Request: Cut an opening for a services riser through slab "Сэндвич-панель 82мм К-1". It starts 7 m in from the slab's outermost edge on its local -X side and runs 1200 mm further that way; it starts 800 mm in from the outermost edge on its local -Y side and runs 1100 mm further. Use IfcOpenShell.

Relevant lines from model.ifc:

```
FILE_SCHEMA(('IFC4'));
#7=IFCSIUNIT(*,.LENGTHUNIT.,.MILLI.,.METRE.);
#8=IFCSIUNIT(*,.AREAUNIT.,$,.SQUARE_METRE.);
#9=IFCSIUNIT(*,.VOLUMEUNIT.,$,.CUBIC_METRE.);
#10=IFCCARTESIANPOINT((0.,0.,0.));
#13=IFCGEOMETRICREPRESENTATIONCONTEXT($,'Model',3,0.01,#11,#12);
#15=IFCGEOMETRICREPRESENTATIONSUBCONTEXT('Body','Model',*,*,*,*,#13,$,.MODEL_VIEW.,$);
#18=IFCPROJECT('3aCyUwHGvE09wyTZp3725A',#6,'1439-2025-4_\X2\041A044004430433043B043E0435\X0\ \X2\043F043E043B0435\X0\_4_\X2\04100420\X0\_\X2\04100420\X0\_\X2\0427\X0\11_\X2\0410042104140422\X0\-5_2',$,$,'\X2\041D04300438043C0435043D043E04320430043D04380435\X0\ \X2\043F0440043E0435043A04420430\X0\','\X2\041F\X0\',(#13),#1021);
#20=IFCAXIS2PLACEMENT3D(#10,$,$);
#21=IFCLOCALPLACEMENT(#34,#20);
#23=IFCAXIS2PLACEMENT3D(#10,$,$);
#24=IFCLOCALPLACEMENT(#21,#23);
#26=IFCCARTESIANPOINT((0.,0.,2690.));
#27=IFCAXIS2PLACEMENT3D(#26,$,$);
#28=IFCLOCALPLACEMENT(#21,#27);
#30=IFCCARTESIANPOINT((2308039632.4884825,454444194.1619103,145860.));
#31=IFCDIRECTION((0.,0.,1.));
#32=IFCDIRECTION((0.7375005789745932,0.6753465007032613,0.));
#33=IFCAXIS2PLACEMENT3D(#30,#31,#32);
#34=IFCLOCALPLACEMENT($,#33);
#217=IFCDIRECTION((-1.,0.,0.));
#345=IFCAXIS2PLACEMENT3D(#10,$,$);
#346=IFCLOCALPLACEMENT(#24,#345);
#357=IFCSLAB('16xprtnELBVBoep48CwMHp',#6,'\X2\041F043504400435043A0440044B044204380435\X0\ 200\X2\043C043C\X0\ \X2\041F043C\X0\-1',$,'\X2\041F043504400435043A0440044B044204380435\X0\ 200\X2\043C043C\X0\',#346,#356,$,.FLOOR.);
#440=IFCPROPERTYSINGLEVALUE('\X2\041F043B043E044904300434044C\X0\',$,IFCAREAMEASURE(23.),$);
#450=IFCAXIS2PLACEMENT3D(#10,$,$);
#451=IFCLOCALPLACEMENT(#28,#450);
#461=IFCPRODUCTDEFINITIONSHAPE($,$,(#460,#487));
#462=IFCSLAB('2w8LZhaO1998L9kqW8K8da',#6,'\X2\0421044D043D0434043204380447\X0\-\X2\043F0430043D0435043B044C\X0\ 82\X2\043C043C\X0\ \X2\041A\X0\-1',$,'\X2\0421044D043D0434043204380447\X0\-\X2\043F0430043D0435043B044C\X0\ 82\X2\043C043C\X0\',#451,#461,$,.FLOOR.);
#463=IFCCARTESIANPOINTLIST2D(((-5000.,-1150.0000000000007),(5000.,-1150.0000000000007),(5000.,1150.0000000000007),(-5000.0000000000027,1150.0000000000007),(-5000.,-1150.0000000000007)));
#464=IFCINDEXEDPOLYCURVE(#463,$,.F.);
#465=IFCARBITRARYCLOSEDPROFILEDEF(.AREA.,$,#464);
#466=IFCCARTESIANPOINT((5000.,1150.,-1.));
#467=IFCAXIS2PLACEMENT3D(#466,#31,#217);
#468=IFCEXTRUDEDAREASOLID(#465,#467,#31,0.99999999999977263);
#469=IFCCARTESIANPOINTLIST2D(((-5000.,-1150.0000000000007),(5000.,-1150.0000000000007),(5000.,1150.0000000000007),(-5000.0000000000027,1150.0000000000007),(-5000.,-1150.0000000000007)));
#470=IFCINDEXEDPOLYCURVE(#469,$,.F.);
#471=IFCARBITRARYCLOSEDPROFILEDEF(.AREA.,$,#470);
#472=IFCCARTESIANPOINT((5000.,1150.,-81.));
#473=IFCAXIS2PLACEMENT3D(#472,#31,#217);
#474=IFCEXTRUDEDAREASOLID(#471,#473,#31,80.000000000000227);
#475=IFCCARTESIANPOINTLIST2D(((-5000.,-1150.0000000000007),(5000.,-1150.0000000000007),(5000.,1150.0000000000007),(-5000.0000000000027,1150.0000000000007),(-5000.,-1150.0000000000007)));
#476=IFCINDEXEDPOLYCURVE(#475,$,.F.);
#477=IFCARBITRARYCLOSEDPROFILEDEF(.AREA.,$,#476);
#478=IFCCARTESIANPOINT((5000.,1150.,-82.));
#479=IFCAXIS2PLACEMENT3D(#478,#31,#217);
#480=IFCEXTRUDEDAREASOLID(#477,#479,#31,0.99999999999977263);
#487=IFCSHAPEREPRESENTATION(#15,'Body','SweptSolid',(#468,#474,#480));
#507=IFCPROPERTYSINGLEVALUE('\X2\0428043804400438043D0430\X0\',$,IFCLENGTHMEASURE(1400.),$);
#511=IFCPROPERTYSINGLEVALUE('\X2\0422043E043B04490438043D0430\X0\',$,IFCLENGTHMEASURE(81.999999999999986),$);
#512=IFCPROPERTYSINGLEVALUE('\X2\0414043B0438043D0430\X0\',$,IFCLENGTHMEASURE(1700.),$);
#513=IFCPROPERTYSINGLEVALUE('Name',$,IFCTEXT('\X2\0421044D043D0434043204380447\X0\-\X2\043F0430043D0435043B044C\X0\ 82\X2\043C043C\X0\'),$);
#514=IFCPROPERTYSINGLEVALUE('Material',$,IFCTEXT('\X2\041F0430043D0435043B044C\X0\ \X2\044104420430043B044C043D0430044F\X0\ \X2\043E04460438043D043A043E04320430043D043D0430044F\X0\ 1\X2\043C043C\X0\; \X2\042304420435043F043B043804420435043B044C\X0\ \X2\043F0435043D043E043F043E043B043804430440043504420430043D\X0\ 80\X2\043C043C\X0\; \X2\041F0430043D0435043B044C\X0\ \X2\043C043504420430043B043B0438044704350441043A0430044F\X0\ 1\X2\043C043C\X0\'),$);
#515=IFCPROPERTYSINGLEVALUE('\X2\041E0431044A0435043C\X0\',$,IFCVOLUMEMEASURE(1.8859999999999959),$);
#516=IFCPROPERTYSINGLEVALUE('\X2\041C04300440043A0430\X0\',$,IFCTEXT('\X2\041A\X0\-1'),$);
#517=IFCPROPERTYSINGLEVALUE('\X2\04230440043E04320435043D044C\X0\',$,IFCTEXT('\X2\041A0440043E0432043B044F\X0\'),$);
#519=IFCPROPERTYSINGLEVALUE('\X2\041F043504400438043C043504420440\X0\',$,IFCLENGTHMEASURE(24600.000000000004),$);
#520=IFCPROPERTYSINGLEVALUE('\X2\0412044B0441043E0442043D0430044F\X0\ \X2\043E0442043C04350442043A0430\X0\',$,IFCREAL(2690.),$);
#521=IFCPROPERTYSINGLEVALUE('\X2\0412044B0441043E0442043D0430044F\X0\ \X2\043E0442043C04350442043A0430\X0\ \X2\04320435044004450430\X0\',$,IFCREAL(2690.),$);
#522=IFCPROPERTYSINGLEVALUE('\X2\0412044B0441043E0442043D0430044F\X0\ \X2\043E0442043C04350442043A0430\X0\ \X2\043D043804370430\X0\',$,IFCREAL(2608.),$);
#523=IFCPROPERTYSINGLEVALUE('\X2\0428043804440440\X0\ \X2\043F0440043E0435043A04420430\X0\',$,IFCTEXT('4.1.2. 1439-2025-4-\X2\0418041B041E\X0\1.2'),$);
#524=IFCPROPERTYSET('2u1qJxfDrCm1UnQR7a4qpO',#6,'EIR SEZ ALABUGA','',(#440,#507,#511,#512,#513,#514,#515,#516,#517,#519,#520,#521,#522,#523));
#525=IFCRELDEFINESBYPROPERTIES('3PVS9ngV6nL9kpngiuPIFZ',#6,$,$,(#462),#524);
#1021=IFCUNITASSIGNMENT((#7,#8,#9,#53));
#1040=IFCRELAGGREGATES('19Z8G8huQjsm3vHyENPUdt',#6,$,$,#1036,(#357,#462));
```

```python
import numpy as np
import ifcopenshell
import ifcopenshell.api.feature
import ifcopenshell.api.geometry
import ifcopenshell.api.pset
import ifcopenshell.api.root
import ifcopenshell.geom
import ifcopenshell.util.element
import ifcopenshell.util.placement
import ifcopenshell.util.representation
import ifcopenshell.util.shape
import ifcopenshell.util.unit

model = ifcopenshell.open("model.ifc")
unit_scale = ifcopenshell.util.unit.calculate_unit_scale(model)
area_scale = ifcopenshell.util.unit.calculate_unit_scale(model, "AREAUNIT")
volume_scale = ifcopenshell.util.unit.calculate_unit_scale(model, "VOLUMEUNIT")
settings = ifcopenshell.geom.settings()


def volume(element):
    """Net volume in cubic metres, openings subtracted."""
    shape = ifcopenshell.geom.create_shape(settings, element)
    return ifcopenshell.util.shape.get_volume(shape.geometry)


slab = model.by_id(462)
before = volume(slab)

# Extent in the slab's own axes, in metres. The edges named are its -X and -Y sides.
slab_shape = ifcopenshell.geom.create_shape(settings, slab)
vertices = ifcopenshell.util.shape.get_vertices(slab_shape.geometry)
x_min, y_min, bottom = vertices.min(axis=0)
top = vertices[:, 2].max()

opening = ifcopenshell.api.root.create_entity(model, ifc_class="IfcOpeningElement", name="Services riser opening", predefined_type="OPENING")
context = ifcopenshell.util.representation.get_context(model, "Model", "Body", "MODEL_VIEW")
width, depth = 1.2, 1.1
outline = [(0.0, 0.0), (width, 0.0), (width, depth), (0.0, depth), (0.0, 0.0)]
# Overshoot both faces by 50 mm so the cut is clean.
shape = ifcopenshell.api.geometry.add_slab_representation(
    model, context=context, depth=top - bottom + 0.1, polyline=outline
)
ifcopenshell.api.geometry.assign_representation(model, product=opening, representation=shape)

matrix = ifcopenshell.util.placement.get_local_placement(slab.ObjectPlacement)
matrix[:, 3] = matrix @ np.append(np.array([x_min + 7, y_min + 0.8, bottom - 0.05]) / unit_scale, 1.0)
ifcopenshell.api.geometry.edit_object_placement(model, product=opening, matrix=matrix, is_si=False)
ifcopenshell.api.feature.add_feature(model, feature=opening, element=slab)

after = volume(slab)

# Update the slab's stored quantities.
pset = model.by_id(ifcopenshell.util.element.get_pset(slab, "EIR SEZ ALABUGA", should_inherit=False)["id"])
ifcopenshell.api.pset.edit_pset(model, pset=pset, properties={
    "Площадь": model.create_entity("IfcAreaMeasure", after / (top - bottom) / area_scale),
    "Объем": model.create_entity("IfcVolumeMeasure", after / volume_scale),
})

print(f"slab volume {before:.3f} -> {after:.3f} m3")

model.write("model_updated.ifc")
```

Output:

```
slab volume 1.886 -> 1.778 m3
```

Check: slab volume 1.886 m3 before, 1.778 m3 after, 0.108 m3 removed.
